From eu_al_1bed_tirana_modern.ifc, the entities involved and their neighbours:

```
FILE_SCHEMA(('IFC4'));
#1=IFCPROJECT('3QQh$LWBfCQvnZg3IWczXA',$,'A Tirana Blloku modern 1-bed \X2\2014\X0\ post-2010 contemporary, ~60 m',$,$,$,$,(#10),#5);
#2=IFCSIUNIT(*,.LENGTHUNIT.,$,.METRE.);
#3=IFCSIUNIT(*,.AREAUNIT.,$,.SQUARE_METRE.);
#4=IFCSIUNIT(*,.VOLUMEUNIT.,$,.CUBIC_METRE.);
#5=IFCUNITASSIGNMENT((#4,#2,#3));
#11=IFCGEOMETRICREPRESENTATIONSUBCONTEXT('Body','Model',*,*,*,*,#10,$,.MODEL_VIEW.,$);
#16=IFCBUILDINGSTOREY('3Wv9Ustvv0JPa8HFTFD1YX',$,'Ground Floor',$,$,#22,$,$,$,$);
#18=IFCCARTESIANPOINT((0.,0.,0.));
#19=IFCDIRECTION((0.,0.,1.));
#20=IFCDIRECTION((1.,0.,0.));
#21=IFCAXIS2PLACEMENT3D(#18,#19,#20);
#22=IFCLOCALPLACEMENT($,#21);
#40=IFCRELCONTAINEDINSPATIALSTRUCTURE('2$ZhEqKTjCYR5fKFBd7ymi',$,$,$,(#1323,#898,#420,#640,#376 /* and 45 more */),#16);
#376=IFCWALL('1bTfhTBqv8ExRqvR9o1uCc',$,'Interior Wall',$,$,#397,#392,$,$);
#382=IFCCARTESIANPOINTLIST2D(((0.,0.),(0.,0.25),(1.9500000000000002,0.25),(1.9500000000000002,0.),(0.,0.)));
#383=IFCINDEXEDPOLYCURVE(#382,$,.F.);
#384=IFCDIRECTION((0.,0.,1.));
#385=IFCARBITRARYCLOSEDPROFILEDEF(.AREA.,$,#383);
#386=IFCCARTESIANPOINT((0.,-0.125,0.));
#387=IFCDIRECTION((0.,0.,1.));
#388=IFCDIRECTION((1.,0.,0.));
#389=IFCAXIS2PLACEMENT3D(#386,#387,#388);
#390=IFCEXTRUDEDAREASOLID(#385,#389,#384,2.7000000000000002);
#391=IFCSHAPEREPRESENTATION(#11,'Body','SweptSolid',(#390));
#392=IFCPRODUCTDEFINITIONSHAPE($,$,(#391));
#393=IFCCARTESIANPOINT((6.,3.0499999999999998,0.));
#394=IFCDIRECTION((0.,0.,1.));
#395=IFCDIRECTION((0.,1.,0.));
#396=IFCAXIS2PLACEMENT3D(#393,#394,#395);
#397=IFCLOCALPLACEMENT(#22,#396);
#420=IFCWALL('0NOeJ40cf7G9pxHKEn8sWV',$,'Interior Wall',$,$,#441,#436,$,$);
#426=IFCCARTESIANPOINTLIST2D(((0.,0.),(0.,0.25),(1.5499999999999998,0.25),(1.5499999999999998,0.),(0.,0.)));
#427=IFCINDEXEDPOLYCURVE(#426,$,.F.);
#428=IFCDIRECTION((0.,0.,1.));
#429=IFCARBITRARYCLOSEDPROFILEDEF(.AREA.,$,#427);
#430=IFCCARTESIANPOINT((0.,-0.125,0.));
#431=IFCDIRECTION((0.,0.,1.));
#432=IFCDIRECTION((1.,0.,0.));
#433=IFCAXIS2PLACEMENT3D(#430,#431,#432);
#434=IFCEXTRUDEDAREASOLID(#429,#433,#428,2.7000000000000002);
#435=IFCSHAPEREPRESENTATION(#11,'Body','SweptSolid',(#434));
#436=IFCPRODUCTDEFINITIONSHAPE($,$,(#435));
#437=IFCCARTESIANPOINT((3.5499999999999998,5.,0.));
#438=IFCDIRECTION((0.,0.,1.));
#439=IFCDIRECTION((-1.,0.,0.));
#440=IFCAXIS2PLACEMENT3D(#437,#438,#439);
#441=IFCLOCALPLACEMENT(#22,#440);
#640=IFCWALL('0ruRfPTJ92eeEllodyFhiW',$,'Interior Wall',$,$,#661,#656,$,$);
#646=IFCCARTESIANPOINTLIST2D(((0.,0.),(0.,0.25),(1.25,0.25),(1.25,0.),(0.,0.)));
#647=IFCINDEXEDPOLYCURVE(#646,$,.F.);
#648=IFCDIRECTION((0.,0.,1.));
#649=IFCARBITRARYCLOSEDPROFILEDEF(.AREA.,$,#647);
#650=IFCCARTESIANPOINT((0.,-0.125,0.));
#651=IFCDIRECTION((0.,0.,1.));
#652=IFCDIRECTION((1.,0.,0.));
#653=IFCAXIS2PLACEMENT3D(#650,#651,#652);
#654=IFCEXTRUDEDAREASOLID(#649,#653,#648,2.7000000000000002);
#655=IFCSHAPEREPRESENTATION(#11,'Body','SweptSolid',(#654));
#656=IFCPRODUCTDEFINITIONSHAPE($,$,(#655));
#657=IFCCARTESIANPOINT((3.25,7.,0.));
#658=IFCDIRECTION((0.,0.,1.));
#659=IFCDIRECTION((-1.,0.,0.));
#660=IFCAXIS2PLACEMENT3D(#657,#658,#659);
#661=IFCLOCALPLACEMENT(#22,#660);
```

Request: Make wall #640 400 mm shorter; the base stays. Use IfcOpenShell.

```python
import ifcopenshell
import ifcopenshell.geom
import ifcopenshell.util.representation
import ifcopenshell.util.shape
import ifcopenshell.util.unit

model = ifcopenshell.open("eu_al_1bed_tirana_modern.ifc")
unit_scale = ifcopenshell.util.unit.calculate_unit_scale(model)
settings = ifcopenshell.geom.settings()


def volume(element):
    """Net volume in cubic metres, openings subtracted."""
    shape = ifcopenshell.geom.create_shape(settings, element)
    return ifcopenshell.util.shape.get_volume(shape.geometry)


wall = model.by_guid("0ruRfPTJ92eeEllodyFhiW")
before = volume(wall)

body = ifcopenshell.util.representation.get_representation(wall, "Model", "Body")
solid = body.Items[0]
old_height = solid.Depth
solid.Depth -= 0.4 / unit_scale
after = volume(wall)

print(f"height {old_height:g} -> {solid.Depth:g}, volume {before:.3f} -> {after:.3f} m3")

model.write("eu_al_1bed_tirana_modern_rev.ifc")
```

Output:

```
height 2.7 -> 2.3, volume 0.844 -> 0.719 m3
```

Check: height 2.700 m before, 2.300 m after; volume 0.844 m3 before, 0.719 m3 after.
